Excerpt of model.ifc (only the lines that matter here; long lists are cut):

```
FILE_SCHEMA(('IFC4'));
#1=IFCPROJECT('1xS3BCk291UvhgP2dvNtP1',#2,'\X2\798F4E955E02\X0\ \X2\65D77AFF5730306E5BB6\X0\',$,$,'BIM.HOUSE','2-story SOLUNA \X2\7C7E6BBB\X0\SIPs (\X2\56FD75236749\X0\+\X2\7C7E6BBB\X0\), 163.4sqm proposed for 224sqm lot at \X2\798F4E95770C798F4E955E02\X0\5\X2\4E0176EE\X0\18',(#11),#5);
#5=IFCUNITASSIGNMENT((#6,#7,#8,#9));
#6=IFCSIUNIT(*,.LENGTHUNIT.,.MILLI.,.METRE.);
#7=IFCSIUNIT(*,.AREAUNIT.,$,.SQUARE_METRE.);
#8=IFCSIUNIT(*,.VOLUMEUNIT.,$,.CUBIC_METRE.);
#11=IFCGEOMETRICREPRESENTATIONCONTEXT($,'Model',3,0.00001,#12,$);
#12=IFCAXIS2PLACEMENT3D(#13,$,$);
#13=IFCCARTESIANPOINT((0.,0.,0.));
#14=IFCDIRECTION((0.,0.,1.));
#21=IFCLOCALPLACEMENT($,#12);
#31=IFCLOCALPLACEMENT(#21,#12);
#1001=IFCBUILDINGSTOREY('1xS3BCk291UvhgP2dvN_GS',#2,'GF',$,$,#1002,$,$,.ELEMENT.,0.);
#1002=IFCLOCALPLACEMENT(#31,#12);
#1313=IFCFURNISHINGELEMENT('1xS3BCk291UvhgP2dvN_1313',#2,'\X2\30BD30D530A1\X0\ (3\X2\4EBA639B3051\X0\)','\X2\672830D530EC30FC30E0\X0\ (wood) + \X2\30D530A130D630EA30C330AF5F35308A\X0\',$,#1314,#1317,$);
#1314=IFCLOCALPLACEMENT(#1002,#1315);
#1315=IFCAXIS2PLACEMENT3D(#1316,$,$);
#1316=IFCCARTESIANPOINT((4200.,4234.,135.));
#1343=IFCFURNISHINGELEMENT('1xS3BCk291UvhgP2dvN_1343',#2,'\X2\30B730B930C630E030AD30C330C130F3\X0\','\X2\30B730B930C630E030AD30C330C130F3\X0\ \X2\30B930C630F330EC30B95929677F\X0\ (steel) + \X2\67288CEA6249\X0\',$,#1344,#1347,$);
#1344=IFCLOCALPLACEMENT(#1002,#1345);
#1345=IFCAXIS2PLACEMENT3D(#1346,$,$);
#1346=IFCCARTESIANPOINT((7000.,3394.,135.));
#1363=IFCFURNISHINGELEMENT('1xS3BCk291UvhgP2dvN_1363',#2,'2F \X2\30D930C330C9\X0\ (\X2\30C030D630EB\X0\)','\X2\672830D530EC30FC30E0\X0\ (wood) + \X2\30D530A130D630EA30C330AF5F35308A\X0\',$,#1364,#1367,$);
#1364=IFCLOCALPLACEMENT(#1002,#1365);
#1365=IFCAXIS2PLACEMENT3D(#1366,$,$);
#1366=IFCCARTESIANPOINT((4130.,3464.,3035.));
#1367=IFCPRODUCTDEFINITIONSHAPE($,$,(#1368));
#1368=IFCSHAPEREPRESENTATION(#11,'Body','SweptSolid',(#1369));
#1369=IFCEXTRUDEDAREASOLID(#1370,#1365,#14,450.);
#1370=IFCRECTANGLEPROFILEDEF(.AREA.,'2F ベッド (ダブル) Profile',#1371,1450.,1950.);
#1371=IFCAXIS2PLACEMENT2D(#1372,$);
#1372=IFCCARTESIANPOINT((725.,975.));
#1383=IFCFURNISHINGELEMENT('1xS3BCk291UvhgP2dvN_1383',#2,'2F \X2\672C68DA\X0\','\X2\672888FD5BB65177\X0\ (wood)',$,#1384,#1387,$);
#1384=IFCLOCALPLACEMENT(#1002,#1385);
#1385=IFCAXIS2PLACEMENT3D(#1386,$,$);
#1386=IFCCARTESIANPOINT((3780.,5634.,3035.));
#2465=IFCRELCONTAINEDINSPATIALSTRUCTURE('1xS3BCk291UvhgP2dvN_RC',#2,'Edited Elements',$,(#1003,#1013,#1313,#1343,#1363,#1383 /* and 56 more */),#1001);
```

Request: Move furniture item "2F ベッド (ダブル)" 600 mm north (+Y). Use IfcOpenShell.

```python
import ifcopenshell
import ifcopenshell.api.geometry
import ifcopenshell.util.placement

model = ifcopenshell.open("model.ifc")

item = model.by_guid("1xS3BCk291UvhgP2dvN_1363")
matrix = ifcopenshell.util.placement.get_local_placement(item.ObjectPlacement)
matrix[1, 3] += 600.0
ifcopenshell.api.geometry.edit_object_placement(model, product=item, matrix=matrix, is_si=False)

print(ifcopenshell.util.placement.get_local_placement(item.ObjectPlacement).round(3) + 0.0)

model.write("model_updated.ifc")
```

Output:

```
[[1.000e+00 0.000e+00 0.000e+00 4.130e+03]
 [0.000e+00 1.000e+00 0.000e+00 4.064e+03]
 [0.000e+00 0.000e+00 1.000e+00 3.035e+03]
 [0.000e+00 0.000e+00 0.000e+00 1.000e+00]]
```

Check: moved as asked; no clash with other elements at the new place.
